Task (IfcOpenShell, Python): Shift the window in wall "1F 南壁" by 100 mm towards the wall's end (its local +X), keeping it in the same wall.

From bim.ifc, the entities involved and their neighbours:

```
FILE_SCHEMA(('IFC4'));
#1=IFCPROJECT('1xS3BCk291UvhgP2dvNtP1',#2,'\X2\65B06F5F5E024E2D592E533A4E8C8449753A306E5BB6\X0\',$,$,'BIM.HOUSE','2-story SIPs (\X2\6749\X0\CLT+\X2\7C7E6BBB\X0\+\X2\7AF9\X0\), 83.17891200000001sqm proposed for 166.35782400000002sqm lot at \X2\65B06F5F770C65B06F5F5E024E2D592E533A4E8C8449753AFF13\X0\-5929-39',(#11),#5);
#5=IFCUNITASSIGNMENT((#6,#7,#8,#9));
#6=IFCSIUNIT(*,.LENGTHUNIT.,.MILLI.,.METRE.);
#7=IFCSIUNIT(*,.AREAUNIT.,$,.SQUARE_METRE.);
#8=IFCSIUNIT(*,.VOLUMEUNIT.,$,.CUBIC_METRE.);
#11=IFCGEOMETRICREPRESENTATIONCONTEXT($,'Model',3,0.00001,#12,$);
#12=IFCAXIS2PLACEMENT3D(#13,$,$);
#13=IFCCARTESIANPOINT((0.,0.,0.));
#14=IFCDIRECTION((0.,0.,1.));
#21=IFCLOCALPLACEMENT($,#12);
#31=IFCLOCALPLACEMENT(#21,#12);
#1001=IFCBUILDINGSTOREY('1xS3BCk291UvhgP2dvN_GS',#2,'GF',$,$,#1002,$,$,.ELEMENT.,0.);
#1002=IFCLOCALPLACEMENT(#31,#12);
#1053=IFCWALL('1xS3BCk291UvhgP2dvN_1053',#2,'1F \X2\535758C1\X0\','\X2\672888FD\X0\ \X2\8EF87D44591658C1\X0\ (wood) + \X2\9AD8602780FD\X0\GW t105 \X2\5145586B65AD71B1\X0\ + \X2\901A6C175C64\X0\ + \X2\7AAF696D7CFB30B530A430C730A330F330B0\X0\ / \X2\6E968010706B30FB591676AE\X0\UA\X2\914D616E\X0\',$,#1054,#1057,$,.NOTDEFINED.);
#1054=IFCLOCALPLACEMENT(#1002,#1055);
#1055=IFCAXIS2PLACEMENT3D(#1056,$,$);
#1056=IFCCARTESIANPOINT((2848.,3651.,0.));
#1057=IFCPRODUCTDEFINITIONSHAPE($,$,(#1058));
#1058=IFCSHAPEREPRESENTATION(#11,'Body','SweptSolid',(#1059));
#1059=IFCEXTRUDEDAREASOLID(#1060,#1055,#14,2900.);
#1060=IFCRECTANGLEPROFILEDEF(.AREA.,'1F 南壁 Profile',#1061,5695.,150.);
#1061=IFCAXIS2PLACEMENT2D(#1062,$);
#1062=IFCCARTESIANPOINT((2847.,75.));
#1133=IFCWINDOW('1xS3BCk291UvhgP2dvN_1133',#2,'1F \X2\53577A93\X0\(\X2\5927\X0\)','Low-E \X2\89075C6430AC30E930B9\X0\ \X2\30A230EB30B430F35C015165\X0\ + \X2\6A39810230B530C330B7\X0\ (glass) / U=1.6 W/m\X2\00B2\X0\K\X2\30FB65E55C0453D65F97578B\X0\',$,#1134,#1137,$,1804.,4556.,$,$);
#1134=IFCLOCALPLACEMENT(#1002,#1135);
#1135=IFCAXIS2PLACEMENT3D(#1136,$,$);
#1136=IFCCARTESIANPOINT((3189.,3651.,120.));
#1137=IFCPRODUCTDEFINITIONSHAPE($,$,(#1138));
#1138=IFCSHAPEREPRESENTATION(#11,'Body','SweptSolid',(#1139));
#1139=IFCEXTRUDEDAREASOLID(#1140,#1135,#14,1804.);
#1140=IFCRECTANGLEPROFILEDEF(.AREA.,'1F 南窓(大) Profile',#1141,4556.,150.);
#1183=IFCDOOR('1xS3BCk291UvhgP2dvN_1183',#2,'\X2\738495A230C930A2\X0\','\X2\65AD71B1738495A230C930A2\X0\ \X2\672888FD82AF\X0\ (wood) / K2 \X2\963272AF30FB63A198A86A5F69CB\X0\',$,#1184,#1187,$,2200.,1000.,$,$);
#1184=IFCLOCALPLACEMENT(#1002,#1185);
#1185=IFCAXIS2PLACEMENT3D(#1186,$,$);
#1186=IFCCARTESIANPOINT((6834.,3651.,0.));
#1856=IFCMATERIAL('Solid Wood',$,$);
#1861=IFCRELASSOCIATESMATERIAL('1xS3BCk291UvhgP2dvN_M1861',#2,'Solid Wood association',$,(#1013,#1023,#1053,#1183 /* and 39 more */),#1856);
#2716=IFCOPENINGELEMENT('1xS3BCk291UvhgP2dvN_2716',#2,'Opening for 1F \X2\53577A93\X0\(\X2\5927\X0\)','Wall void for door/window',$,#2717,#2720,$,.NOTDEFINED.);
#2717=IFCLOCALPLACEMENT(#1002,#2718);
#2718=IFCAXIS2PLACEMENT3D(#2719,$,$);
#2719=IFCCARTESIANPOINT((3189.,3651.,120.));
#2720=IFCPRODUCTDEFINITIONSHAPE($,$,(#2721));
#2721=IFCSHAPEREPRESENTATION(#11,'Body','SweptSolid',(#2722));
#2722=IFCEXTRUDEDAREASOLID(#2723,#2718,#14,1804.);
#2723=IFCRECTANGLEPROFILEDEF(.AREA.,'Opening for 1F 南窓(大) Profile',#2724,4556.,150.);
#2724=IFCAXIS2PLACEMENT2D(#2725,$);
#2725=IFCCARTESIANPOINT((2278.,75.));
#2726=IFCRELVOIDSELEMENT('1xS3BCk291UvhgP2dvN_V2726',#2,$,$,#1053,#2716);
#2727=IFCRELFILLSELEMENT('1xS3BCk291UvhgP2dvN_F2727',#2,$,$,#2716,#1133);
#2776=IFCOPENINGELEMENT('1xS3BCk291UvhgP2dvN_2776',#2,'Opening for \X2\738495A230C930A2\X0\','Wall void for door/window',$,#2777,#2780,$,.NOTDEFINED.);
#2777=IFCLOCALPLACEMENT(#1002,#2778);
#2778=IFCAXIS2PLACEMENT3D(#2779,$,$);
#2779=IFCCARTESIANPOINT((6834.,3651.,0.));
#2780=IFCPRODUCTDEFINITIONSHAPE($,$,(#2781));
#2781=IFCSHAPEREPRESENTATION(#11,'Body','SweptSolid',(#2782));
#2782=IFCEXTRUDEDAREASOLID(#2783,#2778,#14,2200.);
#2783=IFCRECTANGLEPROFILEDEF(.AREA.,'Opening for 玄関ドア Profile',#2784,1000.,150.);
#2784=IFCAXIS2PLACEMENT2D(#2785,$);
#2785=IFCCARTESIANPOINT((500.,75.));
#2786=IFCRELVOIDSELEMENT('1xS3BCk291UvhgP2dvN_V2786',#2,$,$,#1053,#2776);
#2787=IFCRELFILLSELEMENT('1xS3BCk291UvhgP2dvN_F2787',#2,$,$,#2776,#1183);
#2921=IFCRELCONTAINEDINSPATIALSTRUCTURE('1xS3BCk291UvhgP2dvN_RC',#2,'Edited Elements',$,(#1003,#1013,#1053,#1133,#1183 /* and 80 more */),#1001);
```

```python
import ifcopenshell
import ifcopenshell.api.geometry
import ifcopenshell.util.placement

model = ifcopenshell.open("bim.ifc")

window = model.by_id(1133)
opening = window.FillsVoids[0].RelatingOpeningElement
wall = opening.VoidsElements[0].RelatingBuildingElement

wall_matrix = ifcopenshell.util.placement.get_local_placement(wall.ObjectPlacement)
shift = wall_matrix[:3, 0] * 100.0
before = ifcopenshell.util.placement.get_local_placement(window.ObjectPlacement)[:3, 3].copy()

# The window is not placed relative to its opening, so move both.
for product in (opening, window):
    matrix = ifcopenshell.util.placement.get_local_placement(product.ObjectPlacement)
    matrix[:3, 3] += shift
    ifcopenshell.api.geometry.edit_object_placement(model, product=product, matrix=matrix, is_si=False)

after = ifcopenshell.util.placement.get_local_placement(window.ObjectPlacement)[:3, 3]
print("window moved by", (after - before).round(3) + 0.0)

model.write("bim_rev.ifc")
```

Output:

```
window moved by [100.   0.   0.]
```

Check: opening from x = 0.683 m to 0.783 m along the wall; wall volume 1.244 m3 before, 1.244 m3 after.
